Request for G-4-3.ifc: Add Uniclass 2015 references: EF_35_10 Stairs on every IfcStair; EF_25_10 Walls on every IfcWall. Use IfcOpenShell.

First a look at what the model holds.

```python
import ifcopenshell

model = ifcopenshell.open("G-4-3.ifc")
print(model.schema)
print("classifications:", [c.Name for c in model.by_type("IfcClassification")])
for ifc_class in ("IfcDoor", "IfcRoof", "IfcStair", "IfcWall", "IfcWindow"):
    print(ifc_class, len(model.by_type(ifc_class)))
```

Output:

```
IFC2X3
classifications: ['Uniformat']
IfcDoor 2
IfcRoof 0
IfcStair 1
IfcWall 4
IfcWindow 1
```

```python
import ifcopenshell
import ifcopenshell.api.classification

model = ifcopenshell.open("G-4-3.ifc")

# IFC2X3 requires Source and Edition and has no link from the project to the system.
system = model.create_entity("IfcClassification", Source="NBS", Edition="2015", Name="Uniclass 2015")

codes = {
    "IfcStair": ("EF_35_10", "Stairs"),
    "IfcWall": ("EF_25_10", "Walls"),
}
for ifc_class, (code, name) in codes.items():
    products = model.by_type(ifc_class)
    ifcopenshell.api.classification.add_reference(
        model, products=products, classification=system, identification=code, name=name
    )
    print(code, len(products))

model.write("G-4-3_rev.ifc")
```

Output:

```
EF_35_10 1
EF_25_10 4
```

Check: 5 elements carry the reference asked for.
